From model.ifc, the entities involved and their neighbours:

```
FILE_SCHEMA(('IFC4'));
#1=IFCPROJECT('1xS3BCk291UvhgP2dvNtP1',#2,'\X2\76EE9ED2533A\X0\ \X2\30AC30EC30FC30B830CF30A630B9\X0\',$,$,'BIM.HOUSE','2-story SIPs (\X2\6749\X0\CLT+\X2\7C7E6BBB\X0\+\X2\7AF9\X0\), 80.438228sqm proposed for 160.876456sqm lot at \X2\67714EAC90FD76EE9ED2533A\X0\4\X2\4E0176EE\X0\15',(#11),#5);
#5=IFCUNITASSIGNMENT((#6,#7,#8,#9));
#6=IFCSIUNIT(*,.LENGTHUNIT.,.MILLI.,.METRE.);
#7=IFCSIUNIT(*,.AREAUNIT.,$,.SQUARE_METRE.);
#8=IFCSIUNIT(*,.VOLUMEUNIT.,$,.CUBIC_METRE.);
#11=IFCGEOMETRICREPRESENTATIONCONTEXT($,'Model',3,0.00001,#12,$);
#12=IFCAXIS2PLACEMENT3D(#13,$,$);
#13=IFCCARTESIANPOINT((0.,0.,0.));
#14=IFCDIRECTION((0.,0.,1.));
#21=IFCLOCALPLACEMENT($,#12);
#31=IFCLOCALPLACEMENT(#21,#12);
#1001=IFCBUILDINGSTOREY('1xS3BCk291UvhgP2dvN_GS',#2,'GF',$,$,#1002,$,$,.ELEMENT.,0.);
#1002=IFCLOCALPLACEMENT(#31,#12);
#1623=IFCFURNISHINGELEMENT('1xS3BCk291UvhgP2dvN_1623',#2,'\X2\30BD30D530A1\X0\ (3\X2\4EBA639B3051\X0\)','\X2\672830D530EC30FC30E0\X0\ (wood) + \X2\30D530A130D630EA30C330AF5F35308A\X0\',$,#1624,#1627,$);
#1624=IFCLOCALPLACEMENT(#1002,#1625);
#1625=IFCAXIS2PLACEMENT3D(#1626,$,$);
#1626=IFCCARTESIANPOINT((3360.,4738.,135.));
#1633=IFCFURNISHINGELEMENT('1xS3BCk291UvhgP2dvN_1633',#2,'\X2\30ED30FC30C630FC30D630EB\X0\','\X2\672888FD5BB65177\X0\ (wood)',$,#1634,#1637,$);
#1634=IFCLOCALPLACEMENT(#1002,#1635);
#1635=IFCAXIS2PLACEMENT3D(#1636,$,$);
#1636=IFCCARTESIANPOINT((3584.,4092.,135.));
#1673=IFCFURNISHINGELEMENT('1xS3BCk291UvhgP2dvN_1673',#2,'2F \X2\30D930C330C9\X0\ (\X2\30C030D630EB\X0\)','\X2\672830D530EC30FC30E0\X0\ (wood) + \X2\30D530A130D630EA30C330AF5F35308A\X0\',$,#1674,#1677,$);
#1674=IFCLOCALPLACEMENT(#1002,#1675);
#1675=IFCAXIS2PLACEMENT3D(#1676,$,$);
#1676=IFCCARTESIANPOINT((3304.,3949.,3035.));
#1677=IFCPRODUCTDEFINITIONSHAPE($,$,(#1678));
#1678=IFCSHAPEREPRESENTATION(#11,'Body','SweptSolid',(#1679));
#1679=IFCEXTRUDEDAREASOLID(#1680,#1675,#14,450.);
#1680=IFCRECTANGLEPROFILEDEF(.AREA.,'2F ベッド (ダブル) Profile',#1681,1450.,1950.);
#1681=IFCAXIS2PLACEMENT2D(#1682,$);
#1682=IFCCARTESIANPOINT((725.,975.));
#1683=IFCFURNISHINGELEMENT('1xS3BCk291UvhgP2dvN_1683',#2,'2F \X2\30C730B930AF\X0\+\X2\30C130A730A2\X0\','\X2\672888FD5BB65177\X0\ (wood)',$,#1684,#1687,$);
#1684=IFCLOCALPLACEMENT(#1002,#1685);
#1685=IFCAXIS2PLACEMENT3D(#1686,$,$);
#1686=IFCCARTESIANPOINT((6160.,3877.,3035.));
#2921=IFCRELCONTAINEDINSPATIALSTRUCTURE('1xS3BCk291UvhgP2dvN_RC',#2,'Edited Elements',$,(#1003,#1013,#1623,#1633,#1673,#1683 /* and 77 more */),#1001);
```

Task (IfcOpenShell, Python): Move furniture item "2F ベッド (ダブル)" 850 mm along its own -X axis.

```python
import ifcopenshell
import ifcopenshell.api.geometry
import ifcopenshell.util.placement
import ifcopenshell.util.unit

model = ifcopenshell.open("model.ifc")
unit_scale = ifcopenshell.util.unit.calculate_unit_scale(model)

item = model.by_guid("1xS3BCk291UvhgP2dvN_1673")
matrix = ifcopenshell.util.placement.get_local_placement(item.ObjectPlacement)
matrix[:3, 3] -= matrix[:3, 0] * 0.85 / unit_scale
ifcopenshell.api.geometry.edit_object_placement(model, product=item, matrix=matrix, is_si=False)

print(ifcopenshell.util.placement.get_local_placement(item.ObjectPlacement).round(3) + 0.0)

model.write("model-out.ifc")
```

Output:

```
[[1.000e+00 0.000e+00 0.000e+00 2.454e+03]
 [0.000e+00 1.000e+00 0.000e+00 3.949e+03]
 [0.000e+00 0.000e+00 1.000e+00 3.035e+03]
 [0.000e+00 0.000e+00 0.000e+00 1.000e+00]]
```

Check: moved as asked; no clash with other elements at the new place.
